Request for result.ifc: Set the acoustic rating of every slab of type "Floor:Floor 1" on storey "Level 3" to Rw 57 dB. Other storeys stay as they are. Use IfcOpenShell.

First a look at what the model holds.

```python
import ifcopenshell
import ifcopenshell.util.element

model = ifcopenshell.open("result.ifc")
print(model.schema)
storey = next(s for s in model.by_type("IfcBuildingStorey") if s.Name == "Level 3")
slabs = [e for e in ifcopenshell.util.element.get_decomposition(storey) if e.is_a("IfcSlab")]
seen = {}
for e in slabs:
    element_type = ifcopenshell.util.element.get_type(e)
    key = (element_type.Name if element_type != e and element_type else None, ifcopenshell.util.element.get_pset(e, "Pset_SlabCommon", "AcousticRating"))
    seen[key] = seen.get(key, 0) + 1
for (name, value), count in sorted(seen.items(), key=str):
    print(count, "x", name, "|", value)
```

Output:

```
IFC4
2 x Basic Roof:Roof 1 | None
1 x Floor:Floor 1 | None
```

```python
import ifcopenshell
import ifcopenshell.api.pset
import ifcopenshell.util.element

model = ifcopenshell.open("result.ifc")

storey = next(s for s in model.by_type("IfcBuildingStorey") if s.Name == "Level 3")
slabs = [e for e in ifcopenshell.util.element.get_decomposition(storey) if e.is_a("IfcSlab")]

count = 0
for e in slabs:
    element_type = ifcopenshell.util.element.get_type(e)
    if element_type in (None, e) or element_type.Name != "Floor:Floor 1":
        continue
    # add_pset returns the element's existing set when there is one.
    pset = ifcopenshell.api.pset.add_pset(model, product=e, name="Pset_SlabCommon")
    ifcopenshell.api.pset.edit_pset(model, pset=pset, properties={"AcousticRating": "Rw 57 dB"})
    count += 1

print(count, "slabs updated")

model.write("result-out.ifc")
```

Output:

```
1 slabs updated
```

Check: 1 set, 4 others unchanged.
